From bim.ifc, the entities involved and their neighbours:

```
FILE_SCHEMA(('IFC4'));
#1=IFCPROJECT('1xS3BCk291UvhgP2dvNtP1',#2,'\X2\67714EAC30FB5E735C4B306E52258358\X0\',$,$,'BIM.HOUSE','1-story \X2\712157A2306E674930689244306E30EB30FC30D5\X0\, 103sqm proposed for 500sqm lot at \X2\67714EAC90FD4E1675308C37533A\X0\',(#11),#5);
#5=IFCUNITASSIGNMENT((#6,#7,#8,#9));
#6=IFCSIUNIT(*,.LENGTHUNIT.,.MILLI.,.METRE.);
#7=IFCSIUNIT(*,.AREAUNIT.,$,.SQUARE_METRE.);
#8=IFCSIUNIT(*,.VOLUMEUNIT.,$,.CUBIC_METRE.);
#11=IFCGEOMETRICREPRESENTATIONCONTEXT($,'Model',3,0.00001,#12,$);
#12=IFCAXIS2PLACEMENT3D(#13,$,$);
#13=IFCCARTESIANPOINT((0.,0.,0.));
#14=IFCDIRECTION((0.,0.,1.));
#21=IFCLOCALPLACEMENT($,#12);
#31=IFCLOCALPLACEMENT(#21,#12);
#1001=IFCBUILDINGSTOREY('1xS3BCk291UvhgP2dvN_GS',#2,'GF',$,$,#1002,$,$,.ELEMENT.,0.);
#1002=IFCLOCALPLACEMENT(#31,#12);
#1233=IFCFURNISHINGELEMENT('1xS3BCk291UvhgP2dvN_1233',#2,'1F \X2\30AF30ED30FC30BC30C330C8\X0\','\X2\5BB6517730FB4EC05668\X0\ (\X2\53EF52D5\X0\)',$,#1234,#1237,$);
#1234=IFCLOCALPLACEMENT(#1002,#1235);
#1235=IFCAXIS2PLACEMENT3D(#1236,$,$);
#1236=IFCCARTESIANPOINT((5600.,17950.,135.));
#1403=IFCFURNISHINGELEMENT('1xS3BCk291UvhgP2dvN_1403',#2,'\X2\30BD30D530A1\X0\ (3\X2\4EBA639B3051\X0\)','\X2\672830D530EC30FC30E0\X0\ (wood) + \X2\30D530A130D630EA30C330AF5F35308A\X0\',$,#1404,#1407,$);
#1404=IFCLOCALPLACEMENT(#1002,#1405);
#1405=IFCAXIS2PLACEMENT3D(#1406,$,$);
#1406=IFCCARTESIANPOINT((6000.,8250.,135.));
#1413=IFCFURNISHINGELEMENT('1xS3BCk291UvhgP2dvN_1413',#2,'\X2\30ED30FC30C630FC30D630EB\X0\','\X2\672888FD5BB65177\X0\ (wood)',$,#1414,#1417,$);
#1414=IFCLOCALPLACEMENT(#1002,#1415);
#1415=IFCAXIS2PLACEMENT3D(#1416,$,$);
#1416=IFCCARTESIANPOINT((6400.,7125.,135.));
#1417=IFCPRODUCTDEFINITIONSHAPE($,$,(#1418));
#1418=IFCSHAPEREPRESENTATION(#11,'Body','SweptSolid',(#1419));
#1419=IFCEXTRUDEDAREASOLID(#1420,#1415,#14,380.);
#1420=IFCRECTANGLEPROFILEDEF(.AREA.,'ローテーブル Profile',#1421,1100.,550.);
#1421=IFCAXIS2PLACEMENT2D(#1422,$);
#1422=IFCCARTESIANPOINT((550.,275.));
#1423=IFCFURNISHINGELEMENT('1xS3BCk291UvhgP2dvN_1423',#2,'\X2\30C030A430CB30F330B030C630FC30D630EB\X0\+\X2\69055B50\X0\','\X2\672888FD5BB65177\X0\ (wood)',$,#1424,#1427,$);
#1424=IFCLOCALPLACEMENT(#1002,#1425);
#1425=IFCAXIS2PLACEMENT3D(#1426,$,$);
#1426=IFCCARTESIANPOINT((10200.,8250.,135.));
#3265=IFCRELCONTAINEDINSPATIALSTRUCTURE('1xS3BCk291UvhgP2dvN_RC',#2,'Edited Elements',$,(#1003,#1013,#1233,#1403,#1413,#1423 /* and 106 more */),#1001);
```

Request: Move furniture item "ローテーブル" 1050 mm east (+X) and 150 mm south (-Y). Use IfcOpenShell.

```python
import ifcopenshell
import ifcopenshell.api.geometry
import ifcopenshell.util.placement
import ifcopenshell.util.unit

model = ifcopenshell.open("bim.ifc")
unit_scale = ifcopenshell.util.unit.calculate_unit_scale(model)

item = model.by_guid("1xS3BCk291UvhgP2dvN_1413")
matrix = ifcopenshell.util.placement.get_local_placement(item.ObjectPlacement)
matrix[0, 3] += 1.05 / unit_scale
matrix[1, 3] -= 0.15 / unit_scale
ifcopenshell.api.geometry.edit_object_placement(model, product=item, matrix=matrix, is_si=False)

print(ifcopenshell.util.placement.get_local_placement(item.ObjectPlacement).round(3) + 0.0)

model.write("bim_updated.ifc")
```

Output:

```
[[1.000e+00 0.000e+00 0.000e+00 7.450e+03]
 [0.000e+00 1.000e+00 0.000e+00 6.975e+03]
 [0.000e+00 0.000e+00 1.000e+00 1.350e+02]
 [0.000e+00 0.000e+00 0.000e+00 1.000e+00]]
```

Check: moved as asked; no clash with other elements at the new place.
